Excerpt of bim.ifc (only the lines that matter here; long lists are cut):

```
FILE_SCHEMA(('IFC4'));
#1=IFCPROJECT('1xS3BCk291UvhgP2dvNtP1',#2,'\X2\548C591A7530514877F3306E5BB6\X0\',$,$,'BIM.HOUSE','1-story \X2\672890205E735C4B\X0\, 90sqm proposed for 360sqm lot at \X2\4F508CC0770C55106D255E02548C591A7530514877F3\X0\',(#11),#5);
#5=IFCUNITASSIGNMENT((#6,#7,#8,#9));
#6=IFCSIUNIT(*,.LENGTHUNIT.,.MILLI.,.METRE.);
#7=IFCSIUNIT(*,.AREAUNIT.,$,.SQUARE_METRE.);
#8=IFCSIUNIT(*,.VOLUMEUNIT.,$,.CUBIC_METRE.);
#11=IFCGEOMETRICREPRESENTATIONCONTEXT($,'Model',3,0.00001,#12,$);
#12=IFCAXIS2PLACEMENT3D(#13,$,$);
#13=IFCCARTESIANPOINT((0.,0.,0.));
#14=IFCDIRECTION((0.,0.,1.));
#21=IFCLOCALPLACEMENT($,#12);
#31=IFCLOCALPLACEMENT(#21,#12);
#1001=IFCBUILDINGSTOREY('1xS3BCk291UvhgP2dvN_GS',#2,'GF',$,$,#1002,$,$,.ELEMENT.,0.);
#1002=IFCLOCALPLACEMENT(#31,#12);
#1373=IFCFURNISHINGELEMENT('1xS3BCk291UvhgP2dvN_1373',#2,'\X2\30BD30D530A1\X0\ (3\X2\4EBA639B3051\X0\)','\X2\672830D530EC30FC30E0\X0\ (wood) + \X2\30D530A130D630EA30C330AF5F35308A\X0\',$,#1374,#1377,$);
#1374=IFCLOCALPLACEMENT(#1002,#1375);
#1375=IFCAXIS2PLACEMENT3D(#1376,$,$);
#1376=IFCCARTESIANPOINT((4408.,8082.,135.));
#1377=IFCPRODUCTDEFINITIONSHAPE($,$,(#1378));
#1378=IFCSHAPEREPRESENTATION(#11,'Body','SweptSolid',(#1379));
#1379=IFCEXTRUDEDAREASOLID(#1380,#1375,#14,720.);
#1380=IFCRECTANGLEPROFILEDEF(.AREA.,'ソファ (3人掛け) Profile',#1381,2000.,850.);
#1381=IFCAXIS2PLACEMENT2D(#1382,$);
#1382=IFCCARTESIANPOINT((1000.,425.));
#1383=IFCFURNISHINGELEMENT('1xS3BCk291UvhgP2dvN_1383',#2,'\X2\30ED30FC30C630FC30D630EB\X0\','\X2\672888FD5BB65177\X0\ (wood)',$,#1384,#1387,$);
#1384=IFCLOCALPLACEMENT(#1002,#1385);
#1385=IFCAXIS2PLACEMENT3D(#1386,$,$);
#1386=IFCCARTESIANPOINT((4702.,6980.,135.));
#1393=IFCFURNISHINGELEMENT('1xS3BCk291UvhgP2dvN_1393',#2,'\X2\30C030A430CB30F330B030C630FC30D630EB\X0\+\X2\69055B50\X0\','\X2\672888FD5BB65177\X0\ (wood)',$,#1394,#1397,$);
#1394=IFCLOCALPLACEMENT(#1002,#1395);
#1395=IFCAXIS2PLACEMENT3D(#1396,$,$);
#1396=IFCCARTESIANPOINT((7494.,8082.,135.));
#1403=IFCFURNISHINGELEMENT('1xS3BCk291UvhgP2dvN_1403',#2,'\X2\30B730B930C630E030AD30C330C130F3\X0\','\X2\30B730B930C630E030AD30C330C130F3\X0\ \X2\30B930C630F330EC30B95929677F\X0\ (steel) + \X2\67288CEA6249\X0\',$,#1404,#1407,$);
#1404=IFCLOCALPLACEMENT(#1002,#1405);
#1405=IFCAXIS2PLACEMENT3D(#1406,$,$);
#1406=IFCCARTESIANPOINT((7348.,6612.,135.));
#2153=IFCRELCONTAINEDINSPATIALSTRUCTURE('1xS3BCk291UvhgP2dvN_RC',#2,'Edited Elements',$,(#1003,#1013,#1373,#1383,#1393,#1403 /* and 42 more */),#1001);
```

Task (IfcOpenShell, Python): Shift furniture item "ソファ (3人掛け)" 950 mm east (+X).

```python
import ifcopenshell
import ifcopenshell.api.geometry
import ifcopenshell.util.placement
import ifcopenshell.util.unit

model = ifcopenshell.open("bim.ifc")
unit_scale = ifcopenshell.util.unit.calculate_unit_scale(model)

item = model.by_guid("1xS3BCk291UvhgP2dvN_1373")
matrix = ifcopenshell.util.placement.get_local_placement(item.ObjectPlacement)
matrix[0, 3] += 0.95 / unit_scale
ifcopenshell.api.geometry.edit_object_placement(model, product=item, matrix=matrix, is_si=False)

print(ifcopenshell.util.placement.get_local_placement(item.ObjectPlacement).round(3) + 0.0)

model.write("bim-out.ifc")
```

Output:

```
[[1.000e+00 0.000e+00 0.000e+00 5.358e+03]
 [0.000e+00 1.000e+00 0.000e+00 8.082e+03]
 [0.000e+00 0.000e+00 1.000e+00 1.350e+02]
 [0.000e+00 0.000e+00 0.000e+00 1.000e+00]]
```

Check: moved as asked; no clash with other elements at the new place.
